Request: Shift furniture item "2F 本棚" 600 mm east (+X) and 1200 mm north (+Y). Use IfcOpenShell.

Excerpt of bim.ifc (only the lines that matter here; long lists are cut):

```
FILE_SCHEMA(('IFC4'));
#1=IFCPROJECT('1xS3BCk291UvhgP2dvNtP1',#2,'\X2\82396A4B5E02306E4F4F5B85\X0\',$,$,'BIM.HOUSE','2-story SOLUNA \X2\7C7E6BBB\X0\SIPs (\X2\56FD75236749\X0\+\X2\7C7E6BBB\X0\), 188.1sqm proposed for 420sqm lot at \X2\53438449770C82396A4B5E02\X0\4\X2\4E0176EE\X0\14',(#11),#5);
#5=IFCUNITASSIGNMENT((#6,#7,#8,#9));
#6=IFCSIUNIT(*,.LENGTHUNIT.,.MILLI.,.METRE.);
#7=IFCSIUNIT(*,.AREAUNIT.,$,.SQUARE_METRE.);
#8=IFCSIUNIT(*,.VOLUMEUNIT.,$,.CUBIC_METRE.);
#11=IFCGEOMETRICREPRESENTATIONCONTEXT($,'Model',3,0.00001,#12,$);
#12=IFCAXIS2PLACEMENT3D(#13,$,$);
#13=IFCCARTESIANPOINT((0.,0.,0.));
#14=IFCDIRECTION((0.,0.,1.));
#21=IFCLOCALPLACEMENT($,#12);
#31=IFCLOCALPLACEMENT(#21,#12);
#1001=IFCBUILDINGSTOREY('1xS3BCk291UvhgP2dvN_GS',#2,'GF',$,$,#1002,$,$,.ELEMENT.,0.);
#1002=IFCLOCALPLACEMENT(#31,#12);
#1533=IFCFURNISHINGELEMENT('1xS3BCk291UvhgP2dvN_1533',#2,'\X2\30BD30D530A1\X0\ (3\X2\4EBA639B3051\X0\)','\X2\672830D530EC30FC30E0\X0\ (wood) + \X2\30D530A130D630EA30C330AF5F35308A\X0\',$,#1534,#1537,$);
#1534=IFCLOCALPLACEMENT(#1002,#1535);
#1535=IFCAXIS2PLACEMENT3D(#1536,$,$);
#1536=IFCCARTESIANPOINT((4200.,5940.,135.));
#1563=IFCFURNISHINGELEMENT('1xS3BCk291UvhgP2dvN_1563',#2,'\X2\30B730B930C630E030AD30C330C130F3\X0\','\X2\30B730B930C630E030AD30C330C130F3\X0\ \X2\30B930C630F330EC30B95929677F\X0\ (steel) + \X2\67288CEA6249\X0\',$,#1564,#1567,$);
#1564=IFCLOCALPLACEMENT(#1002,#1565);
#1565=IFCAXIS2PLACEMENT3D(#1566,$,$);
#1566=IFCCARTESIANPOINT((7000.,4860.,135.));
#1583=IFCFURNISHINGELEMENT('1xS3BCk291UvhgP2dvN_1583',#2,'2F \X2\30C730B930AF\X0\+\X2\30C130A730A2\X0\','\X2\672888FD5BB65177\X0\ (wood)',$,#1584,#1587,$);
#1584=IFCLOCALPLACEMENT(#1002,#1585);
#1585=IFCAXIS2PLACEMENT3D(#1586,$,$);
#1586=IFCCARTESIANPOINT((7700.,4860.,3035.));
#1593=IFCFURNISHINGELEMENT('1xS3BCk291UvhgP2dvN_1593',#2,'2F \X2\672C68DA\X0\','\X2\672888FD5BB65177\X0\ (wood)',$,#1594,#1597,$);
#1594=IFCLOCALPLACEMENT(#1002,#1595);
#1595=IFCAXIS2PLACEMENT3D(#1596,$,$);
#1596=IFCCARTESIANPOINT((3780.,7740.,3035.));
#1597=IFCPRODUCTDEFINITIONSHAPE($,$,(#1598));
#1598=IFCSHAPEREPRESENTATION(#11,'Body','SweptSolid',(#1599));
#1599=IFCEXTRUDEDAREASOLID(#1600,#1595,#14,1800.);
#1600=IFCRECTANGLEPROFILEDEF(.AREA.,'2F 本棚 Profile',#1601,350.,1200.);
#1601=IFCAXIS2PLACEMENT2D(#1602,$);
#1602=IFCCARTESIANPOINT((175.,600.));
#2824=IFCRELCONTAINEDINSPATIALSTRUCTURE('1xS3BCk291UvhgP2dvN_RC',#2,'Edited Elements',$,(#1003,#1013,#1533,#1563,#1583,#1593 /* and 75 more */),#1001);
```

```python
import ifcopenshell
import ifcopenshell.api.geometry
import ifcopenshell.util.placement
import ifcopenshell.util.unit

model = ifcopenshell.open("bim.ifc")
unit_scale = ifcopenshell.util.unit.calculate_unit_scale(model)

item = model.by_guid("1xS3BCk291UvhgP2dvN_1593")
matrix = ifcopenshell.util.placement.get_local_placement(item.ObjectPlacement)
matrix[0, 3] += 0.6 / unit_scale
matrix[1, 3] += 1.2 / unit_scale
ifcopenshell.api.geometry.edit_object_placement(model, product=item, matrix=matrix, is_si=False)

print(ifcopenshell.util.placement.get_local_placement(item.ObjectPlacement).round(3) + 0.0)

model.write("bim_updated.ifc")
```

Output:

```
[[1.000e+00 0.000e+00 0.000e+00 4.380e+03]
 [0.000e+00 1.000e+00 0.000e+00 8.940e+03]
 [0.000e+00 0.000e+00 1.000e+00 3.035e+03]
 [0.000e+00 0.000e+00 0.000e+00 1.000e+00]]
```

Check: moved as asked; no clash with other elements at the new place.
